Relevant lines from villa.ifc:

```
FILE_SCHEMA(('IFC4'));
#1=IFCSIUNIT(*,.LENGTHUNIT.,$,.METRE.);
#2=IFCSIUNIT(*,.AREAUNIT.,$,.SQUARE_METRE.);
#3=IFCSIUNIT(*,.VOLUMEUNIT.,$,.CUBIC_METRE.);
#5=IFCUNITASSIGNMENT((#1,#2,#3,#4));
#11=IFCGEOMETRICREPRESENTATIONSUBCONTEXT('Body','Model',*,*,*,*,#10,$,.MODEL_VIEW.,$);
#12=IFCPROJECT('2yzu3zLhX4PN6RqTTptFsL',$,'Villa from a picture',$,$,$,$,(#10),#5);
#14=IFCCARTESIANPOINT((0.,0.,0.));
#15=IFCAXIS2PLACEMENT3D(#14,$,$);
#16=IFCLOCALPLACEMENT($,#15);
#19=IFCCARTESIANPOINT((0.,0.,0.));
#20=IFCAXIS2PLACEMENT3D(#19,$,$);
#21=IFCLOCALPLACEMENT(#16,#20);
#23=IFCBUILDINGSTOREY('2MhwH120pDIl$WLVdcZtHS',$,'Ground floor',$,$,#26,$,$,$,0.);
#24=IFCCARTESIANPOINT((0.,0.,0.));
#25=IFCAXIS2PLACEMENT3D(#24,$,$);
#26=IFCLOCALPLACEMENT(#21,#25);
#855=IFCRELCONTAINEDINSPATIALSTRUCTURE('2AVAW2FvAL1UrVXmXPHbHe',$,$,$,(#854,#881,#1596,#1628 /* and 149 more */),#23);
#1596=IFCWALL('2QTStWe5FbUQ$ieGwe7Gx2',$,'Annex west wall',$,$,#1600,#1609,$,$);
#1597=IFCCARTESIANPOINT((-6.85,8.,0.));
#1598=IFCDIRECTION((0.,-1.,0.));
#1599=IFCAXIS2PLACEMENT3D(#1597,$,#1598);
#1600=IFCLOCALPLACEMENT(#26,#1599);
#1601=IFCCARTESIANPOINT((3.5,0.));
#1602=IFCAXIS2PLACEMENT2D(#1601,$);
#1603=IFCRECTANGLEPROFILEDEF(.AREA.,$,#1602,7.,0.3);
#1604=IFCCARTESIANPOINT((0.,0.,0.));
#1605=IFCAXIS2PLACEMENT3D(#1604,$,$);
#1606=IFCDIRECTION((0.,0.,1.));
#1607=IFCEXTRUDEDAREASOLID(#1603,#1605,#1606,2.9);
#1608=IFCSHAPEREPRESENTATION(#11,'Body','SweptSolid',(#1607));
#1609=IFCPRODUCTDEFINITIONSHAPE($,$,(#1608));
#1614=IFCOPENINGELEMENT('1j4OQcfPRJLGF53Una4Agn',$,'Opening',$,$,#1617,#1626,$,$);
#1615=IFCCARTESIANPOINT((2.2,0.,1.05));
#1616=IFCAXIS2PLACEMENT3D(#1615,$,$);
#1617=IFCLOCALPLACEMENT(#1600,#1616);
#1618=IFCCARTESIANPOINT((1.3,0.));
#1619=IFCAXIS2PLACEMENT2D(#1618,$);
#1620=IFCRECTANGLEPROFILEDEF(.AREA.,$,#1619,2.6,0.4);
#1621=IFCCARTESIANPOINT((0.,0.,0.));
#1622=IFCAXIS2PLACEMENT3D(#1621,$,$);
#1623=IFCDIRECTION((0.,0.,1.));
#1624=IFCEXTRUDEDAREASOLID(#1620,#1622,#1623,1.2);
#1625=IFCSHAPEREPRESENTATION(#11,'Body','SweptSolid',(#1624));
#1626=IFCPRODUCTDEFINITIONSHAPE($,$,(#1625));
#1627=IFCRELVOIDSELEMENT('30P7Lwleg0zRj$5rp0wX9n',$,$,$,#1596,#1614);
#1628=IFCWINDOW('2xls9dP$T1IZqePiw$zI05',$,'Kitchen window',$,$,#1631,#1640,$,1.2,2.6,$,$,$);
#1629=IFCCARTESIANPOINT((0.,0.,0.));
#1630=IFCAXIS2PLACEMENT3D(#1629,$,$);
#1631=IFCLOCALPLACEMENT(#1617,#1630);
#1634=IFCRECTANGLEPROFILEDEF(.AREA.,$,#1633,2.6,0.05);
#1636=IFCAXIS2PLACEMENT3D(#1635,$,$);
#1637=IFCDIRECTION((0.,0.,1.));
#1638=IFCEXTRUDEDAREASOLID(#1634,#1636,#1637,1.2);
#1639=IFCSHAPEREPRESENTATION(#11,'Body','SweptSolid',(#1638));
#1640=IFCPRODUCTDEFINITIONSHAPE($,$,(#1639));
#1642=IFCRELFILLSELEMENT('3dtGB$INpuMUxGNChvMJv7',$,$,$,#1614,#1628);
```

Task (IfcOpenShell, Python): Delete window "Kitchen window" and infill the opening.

```python
import ifcopenshell
import ifcopenshell.api.feature
import ifcopenshell.api.root
import ifcopenshell.geom
import ifcopenshell.util.shape

model = ifcopenshell.open("villa.ifc")
settings = ifcopenshell.geom.settings()


def volume(element):
    """Net volume in cubic metres, openings subtracted."""
    shape = ifcopenshell.geom.create_shape(settings, element)
    return ifcopenshell.util.shape.get_volume(shape.geometry)


window = model.by_guid("2xls9dP$T1IZqePiw$zI05")
opening = window.FillsVoids[0].RelatingOpeningElement
wall = opening.VoidsElements[0].RelatingBuildingElement
before = volume(wall)

ifcopenshell.api.root.remove_product(model, product=window)
ifcopenshell.api.feature.remove_feature(model, feature=opening)

after = volume(wall)

print(f"wall volume {before:.3f} -> {after:.3f} m3")

model.write("villa_edited.ifc")
```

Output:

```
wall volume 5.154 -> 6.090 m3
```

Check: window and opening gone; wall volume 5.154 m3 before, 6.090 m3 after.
